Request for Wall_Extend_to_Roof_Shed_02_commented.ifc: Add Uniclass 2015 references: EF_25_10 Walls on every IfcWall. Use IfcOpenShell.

First a look at what the model holds.

```python
import ifcopenshell

model = ifcopenshell.open("Wall_Extend_to_Roof_Shed_02_commented.ifc")
print(model.schema)
print("classifications:", [c.Name for c in model.by_type("IfcClassification")])
for ifc_class in ("IfcDoor", "IfcRoof", "IfcStair", "IfcWall", "IfcWindow"):
    print(ifc_class, len(model.by_type(ifc_class)))
```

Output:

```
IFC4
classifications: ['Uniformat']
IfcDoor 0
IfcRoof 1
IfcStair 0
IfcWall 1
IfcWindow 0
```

```python
import ifcopenshell
import ifcopenshell.api.classification

model = ifcopenshell.open("Wall_Extend_to_Roof_Shed_02_commented.ifc")

system = ifcopenshell.api.classification.add_classification(model, classification="Uniclass 2015")

codes = {
    "IfcWall": ("EF_25_10", "Walls"),
}
for ifc_class, (code, name) in codes.items():
    products = model.by_type(ifc_class)
    ifcopenshell.api.classification.add_reference(
        model, products=products, classification=system, identification=code, name=name
    )
    print(code, len(products))

model.write("Wall_Extend_to_Roof_Shed_02_commented_edited.ifc")
```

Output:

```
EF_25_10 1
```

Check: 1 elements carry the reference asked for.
